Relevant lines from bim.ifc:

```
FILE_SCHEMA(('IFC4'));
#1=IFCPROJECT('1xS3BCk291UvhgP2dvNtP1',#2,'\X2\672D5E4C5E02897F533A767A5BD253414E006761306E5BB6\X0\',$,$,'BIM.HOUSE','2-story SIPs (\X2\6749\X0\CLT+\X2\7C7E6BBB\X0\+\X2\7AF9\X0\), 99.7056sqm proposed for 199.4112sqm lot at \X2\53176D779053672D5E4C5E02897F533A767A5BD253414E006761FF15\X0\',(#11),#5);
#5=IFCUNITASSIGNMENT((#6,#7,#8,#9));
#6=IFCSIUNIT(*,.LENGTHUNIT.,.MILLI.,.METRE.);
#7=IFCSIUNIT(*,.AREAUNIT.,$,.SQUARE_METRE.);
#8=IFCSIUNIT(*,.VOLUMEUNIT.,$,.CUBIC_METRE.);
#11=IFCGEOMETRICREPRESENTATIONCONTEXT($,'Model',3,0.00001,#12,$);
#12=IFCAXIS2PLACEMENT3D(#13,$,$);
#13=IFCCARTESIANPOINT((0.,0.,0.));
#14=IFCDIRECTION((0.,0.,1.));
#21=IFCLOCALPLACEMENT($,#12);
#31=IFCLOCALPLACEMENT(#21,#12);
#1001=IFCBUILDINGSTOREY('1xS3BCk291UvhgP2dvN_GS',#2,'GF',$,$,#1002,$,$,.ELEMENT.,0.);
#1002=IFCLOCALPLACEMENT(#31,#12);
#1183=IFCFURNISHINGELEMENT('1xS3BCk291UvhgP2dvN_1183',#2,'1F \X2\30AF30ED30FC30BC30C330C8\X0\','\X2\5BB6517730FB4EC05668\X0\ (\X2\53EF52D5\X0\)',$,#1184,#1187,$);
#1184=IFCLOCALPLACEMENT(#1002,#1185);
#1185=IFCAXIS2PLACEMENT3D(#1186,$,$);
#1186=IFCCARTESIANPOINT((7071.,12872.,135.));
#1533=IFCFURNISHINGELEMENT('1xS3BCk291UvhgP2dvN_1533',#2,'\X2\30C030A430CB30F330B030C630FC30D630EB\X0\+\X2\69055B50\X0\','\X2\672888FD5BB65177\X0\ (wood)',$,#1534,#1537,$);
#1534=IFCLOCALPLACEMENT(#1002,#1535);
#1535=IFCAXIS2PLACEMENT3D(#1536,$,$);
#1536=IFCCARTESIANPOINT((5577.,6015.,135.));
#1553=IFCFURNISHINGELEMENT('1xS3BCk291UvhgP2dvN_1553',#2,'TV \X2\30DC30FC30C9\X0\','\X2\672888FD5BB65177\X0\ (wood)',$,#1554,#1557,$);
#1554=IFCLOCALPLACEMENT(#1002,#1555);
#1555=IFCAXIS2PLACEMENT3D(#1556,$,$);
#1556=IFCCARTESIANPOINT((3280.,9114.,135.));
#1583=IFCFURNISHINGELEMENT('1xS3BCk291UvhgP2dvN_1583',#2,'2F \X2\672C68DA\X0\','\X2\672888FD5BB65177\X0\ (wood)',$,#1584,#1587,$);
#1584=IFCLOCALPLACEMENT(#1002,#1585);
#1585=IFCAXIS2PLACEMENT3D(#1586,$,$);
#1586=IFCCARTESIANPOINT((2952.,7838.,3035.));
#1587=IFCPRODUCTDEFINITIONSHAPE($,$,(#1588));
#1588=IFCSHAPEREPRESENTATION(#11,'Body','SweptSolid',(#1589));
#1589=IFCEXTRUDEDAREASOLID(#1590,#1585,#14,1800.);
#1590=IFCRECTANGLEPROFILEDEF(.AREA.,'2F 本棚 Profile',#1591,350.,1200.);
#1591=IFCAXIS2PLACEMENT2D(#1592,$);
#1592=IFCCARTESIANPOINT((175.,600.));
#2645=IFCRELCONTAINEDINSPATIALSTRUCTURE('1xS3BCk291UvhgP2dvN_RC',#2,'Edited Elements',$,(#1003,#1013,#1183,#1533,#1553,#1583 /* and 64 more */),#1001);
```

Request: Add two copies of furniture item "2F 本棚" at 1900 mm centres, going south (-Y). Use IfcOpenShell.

```python
import numpy as np
import ifcopenshell
import ifcopenshell.api.geometry
import ifcopenshell.api.root
import ifcopenshell.util.element
import ifcopenshell.util.placement

model = ifcopenshell.open("bim.ifc")


def reuse_history(source, copy):
    """copy_class also copies each property set's owner history, people and application; keep the originals."""
    for rel in copy.IsDefinedBy:
        if rel.is_a("IfcRelDefinesByProperties") and (history := rel.RelatingPropertyDefinition.OwnerHistory):
            rel.RelatingPropertyDefinition.OwnerHistory = source.OwnerHistory
            ifcopenshell.util.element.remove_deep2(model, history)


source = model.by_guid("1xS3BCk291UvhgP2dvN_1583")
base = ifcopenshell.util.placement.get_local_placement(source.ObjectPlacement)
step = np.array([0.0, -1.0, 0.0]) * 1900.0

for i in range(1, 3):
    copy = ifcopenshell.api.root.copy_class(model, product=source)
    copy.Representation = ifcopenshell.util.element.copy_deep(
        model, source.Representation, exclude=["IfcGeometricRepresentationContext", "IfcRepresentationMap"]
    )
    reuse_history(source, copy)
    matrix = base.copy()
    matrix[:3, 3] += i * step
    print("added at", matrix[:3, 3].round(3) + 0.0)
    ifcopenshell.api.geometry.edit_object_placement(model, product=copy, matrix=matrix, is_si=False)

model.write("bim_v2.ifc")
```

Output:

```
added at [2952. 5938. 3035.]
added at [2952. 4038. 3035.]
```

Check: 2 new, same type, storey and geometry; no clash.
